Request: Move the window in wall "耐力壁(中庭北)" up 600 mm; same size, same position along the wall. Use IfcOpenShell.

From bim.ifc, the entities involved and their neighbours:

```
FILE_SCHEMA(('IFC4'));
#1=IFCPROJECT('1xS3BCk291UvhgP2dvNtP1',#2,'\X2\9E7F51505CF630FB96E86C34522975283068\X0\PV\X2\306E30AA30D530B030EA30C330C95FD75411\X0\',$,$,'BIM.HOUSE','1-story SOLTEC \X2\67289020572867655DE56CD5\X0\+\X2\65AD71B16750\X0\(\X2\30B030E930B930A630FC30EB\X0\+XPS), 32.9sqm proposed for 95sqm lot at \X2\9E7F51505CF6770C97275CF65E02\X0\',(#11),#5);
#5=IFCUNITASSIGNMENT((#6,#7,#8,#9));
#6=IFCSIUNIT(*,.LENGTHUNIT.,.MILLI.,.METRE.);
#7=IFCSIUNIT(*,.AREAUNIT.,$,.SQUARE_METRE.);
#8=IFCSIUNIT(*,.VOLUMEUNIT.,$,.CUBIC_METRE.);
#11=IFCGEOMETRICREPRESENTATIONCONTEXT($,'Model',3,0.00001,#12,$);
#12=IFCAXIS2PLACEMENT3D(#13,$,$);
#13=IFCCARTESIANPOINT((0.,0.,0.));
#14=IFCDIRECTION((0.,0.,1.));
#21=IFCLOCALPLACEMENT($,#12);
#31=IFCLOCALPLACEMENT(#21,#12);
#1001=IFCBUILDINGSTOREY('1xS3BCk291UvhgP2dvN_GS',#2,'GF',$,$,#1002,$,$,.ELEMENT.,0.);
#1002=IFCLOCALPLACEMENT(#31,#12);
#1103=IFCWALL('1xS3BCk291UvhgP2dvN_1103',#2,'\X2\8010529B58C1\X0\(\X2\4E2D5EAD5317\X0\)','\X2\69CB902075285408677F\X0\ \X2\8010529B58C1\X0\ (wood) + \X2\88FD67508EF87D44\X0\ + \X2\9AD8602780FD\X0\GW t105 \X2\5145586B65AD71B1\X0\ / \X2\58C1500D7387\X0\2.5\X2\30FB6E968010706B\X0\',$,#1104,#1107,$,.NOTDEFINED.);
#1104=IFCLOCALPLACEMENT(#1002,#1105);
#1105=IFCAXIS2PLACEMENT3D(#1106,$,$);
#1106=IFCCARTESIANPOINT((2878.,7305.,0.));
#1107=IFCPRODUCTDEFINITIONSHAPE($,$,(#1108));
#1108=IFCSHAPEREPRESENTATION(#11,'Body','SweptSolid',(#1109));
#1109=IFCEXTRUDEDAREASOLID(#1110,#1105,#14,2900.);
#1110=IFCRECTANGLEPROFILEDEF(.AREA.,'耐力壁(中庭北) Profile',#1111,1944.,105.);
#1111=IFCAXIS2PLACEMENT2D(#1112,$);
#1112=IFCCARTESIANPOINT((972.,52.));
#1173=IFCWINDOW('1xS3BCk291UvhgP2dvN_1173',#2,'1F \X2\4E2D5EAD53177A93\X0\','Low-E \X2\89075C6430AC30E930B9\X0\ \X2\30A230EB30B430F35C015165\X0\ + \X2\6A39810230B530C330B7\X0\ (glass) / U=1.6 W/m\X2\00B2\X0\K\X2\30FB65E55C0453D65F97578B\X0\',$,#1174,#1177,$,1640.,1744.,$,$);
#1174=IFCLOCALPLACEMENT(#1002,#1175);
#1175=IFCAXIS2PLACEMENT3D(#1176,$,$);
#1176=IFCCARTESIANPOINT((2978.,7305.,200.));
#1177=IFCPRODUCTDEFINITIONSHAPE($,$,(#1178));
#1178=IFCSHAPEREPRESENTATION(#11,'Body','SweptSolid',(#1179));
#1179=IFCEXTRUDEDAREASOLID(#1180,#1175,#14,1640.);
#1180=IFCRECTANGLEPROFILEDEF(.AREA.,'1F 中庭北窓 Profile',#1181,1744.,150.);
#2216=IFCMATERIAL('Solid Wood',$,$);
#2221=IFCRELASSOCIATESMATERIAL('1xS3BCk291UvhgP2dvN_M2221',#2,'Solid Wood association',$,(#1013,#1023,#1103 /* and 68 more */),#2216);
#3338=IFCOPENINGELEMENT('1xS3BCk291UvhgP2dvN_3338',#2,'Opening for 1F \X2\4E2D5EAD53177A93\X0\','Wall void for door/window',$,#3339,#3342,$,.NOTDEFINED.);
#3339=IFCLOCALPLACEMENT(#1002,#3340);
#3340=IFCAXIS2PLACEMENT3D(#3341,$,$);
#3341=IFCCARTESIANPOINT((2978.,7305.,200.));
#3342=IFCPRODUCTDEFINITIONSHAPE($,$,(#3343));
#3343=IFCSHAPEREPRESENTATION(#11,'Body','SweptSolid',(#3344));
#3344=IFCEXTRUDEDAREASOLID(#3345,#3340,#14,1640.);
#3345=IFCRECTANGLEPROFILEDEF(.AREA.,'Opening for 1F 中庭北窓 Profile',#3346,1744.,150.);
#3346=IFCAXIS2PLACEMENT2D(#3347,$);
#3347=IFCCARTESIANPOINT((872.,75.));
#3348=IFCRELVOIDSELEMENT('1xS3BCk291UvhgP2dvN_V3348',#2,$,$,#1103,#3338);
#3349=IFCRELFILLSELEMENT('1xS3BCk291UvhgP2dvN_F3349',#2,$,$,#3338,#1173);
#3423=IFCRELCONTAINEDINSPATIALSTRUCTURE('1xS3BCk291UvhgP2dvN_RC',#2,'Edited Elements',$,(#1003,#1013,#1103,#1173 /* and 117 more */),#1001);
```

```python
import numpy as np
import ifcopenshell
import ifcopenshell.api.geometry
import ifcopenshell.util.placement
import ifcopenshell.util.unit

model = ifcopenshell.open("bim.ifc")
unit_scale = ifcopenshell.util.unit.calculate_unit_scale(model)

window = model.by_guid("1xS3BCk291UvhgP2dvN_1173")
opening = window.FillsVoids[0].RelatingOpeningElement
dz = 600.0

shift = np.array([0.0, 0.0, dz])
# The window is not placed relative to its opening, so move both.
for product in (opening, window):
    matrix = ifcopenshell.util.placement.get_local_placement(product.ObjectPlacement)
    matrix[:3, 3] += shift
    ifcopenshell.api.geometry.edit_object_placement(model, product=product, matrix=matrix, is_si=False)

print(f"moved by {dz * unit_scale:+.3f} m")

model.write("bim_updated.ifc")
```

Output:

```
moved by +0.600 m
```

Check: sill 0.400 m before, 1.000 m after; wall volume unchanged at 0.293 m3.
